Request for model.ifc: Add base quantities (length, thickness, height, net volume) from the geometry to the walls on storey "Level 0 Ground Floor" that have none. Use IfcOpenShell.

First a look at what the model holds.

```python
import ifcopenshell
import ifcopenshell.util.element
import ifcopenshell.util.unit

model = ifcopenshell.open("model.ifc")
print(model.schema)
for unit_type in ("LENGTHUNIT", "AREAUNIT", "VOLUMEUNIT"):
    print(unit_type, ifcopenshell.util.unit.calculate_unit_scale(model, unit_type))
storey = next(s for s in model.by_type("IfcBuildingStorey") if s.Name == "Level 0 Ground Floor")
walls = [e for e in ifcopenshell.util.element.get_decomposition(storey) if e.is_a("IfcWall")]
for e in sorted(walls, key=lambda e: e.id()):
    print(e.id(), e.is_a(), e.Name, list(ifcopenshell.util.element.get_psets(e, qtos_only=True)), sep=" | ")
```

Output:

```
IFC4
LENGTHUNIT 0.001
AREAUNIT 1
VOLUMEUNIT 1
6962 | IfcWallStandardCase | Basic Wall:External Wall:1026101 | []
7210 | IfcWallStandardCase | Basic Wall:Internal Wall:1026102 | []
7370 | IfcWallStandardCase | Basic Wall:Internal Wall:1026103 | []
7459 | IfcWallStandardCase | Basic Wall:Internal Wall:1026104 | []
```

```python
import ifcopenshell
import ifcopenshell.api.pset
import ifcopenshell.geom
import ifcopenshell.util.element
import ifcopenshell.util.shape
import ifcopenshell.util.unit

model = ifcopenshell.open("model.ifc")
unit_scale = ifcopenshell.util.unit.calculate_unit_scale(model)
volume_scale = ifcopenshell.util.unit.calculate_unit_scale(model, "VOLUMEUNIT")
settings = ifcopenshell.geom.settings()

storey = next(s for s in model.by_type("IfcBuildingStorey") if s.Name == "Level 0 Ground Floor")
walls = [e for e in ifcopenshell.util.element.get_decomposition(storey) if e.is_a("IfcWall")]

for e in sorted(walls, key=lambda e: e.id()):
    if ifcopenshell.util.element.get_psets(e, qtos_only=True, should_inherit=False):
        continue
    # Geometry comes back in metres, in the element's own axes.
    shape = ifcopenshell.geom.create_shape(settings, e)
    values = {
        "Length": ifcopenshell.util.shape.get_x(shape.geometry) / unit_scale,
        "Width": ifcopenshell.util.shape.get_y(shape.geometry) / unit_scale,
        "Height": ifcopenshell.util.shape.get_z(shape.geometry) / unit_scale,
        "NetVolume": ifcopenshell.util.shape.get_volume(shape.geometry) / volume_scale,
    }
    qto = ifcopenshell.api.pset.add_qto(model, product=e, name="Qto_WallBaseQuantities")
    ifcopenshell.api.pset.edit_qto(model, qto=qto, properties=values)
    print(e.id(), {k: round(v, 3) for k, v in values.items()})

model.write("model_edited.ifc")
```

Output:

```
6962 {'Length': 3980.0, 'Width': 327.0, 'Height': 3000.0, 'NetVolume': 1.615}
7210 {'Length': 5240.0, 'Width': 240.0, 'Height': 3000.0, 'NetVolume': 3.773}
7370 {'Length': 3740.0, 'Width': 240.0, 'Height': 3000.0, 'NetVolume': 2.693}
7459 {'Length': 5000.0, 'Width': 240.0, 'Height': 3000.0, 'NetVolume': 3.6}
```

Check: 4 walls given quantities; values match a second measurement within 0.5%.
